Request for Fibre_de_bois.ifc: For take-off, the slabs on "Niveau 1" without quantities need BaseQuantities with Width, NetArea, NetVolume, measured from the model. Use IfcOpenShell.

First a look at what the model holds.

```python
import ifcopenshell
import ifcopenshell.util.element
import ifcopenshell.util.unit

model = ifcopenshell.open("Fibre_de_bois.ifc")
print(model.schema)
for unit_type in ("LENGTHUNIT", "AREAUNIT", "VOLUMEUNIT"):
    print(unit_type, ifcopenshell.util.unit.calculate_unit_scale(model, unit_type))
storey = next(s for s in model.by_type("IfcBuildingStorey") if s.Name == "Niveau 1")
slabs = [e for e in ifcopenshell.util.element.get_decomposition(storey) if e.is_a("IfcSlab")]
for e in sorted(slabs, key=lambda e: e.id()):
    print(e.id(), e.is_a(), e.Name, list(ifcopenshell.util.element.get_psets(e, qtos_only=True)), sep=" | ")
```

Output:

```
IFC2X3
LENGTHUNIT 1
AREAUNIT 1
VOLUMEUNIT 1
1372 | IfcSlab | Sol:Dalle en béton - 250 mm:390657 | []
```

```python
import ifcopenshell
import ifcopenshell.api.pset
import ifcopenshell.geom
import ifcopenshell.util.element
import ifcopenshell.util.shape
import ifcopenshell.util.unit

model = ifcopenshell.open("Fibre_de_bois.ifc")
unit_scale = ifcopenshell.util.unit.calculate_unit_scale(model)
area_scale = ifcopenshell.util.unit.calculate_unit_scale(model, "AREAUNIT")
volume_scale = ifcopenshell.util.unit.calculate_unit_scale(model, "VOLUMEUNIT")
settings = ifcopenshell.geom.settings()

storey = next(s for s in model.by_type("IfcBuildingStorey") if s.Name == "Niveau 1")
slabs = [e for e in ifcopenshell.util.element.get_decomposition(storey) if e.is_a("IfcSlab")]

for e in sorted(slabs, key=lambda e: e.id()):
    if ifcopenshell.util.element.get_psets(e, qtos_only=True, should_inherit=False):
        continue
    # Geometry comes back in metres, in the element's own axes.
    shape = ifcopenshell.geom.create_shape(settings, e)
    values = {
        "Width": ifcopenshell.util.shape.get_z(shape.geometry) / unit_scale,
        "NetArea": ifcopenshell.util.shape.get_footprint_area(shape.geometry) / area_scale,
        "NetVolume": ifcopenshell.util.shape.get_volume(shape.geometry) / volume_scale,
    }
    qto = ifcopenshell.api.pset.add_qto(model, product=e, name="BaseQuantities")
    ifcopenshell.api.pset.edit_qto(model, qto=qto, properties=values)
    print(e.id(), {k: round(v, 3) for k, v in values.items()})

model.write("Fibre_de_bois_rev.ifc")
```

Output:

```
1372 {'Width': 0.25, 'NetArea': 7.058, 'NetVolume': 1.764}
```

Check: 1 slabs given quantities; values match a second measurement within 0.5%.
